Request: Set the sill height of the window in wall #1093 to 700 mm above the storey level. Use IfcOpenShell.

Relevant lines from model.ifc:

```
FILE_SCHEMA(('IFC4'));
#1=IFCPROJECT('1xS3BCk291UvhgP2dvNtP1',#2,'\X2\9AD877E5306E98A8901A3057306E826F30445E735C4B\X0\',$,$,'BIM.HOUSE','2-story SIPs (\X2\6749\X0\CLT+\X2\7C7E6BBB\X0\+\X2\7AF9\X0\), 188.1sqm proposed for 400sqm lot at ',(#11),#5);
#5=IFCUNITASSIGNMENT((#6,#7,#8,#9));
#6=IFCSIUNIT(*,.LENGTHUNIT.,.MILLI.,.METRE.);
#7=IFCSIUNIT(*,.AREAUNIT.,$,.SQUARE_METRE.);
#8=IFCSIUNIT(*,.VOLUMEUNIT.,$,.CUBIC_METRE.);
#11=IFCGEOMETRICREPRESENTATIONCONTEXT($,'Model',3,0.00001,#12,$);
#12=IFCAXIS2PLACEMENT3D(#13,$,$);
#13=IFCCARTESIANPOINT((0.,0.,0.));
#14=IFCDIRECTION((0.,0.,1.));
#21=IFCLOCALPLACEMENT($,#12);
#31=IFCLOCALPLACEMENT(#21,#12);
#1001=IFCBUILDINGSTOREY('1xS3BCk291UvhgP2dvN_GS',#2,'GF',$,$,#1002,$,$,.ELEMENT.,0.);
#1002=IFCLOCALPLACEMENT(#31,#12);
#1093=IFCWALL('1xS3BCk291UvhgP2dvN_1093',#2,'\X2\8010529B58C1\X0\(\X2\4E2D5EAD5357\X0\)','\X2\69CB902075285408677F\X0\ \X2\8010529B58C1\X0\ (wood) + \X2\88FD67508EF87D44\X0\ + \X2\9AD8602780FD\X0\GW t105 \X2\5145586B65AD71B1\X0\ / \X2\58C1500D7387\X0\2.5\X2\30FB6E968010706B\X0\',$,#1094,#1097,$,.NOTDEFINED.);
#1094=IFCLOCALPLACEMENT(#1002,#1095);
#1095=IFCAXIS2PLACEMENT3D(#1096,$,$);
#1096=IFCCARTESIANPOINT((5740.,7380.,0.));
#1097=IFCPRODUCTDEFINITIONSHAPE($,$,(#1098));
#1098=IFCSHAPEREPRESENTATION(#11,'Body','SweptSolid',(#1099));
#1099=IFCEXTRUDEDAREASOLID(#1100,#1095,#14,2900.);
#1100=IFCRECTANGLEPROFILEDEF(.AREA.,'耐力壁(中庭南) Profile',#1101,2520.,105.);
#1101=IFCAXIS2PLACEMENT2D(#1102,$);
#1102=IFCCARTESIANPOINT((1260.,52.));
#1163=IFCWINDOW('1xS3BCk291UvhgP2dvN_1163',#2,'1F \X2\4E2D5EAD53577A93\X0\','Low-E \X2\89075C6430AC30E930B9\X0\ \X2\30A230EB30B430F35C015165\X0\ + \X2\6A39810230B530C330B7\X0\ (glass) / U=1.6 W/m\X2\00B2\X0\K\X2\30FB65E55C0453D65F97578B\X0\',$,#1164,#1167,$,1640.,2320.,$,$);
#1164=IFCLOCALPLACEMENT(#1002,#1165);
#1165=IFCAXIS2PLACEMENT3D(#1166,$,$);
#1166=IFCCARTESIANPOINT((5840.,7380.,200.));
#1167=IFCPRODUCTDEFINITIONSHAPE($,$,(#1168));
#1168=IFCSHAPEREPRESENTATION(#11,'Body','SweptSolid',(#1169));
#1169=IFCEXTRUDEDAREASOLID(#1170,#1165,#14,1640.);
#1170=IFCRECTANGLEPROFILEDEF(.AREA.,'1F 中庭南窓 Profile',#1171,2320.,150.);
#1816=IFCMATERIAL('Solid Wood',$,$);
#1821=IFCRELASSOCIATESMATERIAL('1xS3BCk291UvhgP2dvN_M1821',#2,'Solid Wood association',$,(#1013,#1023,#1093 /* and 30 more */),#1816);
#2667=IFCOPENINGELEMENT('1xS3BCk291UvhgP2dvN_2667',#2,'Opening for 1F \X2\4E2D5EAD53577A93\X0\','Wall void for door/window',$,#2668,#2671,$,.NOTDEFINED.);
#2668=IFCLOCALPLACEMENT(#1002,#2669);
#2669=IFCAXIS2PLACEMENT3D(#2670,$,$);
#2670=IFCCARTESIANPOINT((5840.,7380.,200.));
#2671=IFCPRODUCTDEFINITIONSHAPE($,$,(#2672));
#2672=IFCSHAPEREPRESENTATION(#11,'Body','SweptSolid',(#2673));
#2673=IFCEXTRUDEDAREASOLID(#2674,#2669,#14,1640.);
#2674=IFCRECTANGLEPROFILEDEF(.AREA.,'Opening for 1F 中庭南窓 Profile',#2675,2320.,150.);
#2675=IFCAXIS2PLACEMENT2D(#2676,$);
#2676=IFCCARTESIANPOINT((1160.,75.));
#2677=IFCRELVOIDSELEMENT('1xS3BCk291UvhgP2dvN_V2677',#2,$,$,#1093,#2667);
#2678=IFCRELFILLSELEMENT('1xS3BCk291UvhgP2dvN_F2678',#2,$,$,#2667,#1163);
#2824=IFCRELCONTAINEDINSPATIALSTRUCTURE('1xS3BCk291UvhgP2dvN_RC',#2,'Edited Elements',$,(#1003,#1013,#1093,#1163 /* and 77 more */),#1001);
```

```python
import numpy as np
import ifcopenshell
import ifcopenshell.api.geometry
import ifcopenshell.geom
import ifcopenshell.util.element
import ifcopenshell.util.placement
import ifcopenshell.util.shape
import ifcopenshell.util.unit

model = ifcopenshell.open("model.ifc")
unit_scale = ifcopenshell.util.unit.calculate_unit_scale(model)

window = model.by_guid("1xS3BCk291UvhgP2dvN_1163")
opening = window.FillsVoids[0].RelatingOpeningElement
storey = ifcopenshell.util.element.get_container(window, ifc_class="IfcBuildingStorey")
level = ifcopenshell.util.placement.get_local_placement(storey.ObjectPlacement)[2, 3]

# The opening's origin need not be at the sill, so measure its lowest point.
shape = ifcopenshell.geom.create_shape(ifcopenshell.geom.settings(), opening)
bottom = ifcopenshell.util.shape.get_shape_bottom_elevation(shape, shape.geometry) / unit_scale
dz = level + 0.7 / unit_scale - bottom

shift = np.array([0.0, 0.0, dz])
# The window is not placed relative to its opening, so move both.
for product in (opening, window):
    matrix = ifcopenshell.util.placement.get_local_placement(product.ObjectPlacement)
    matrix[:3, 3] += shift
    ifcopenshell.api.geometry.edit_object_placement(model, product=product, matrix=matrix, is_si=False)

print(f"moved by {dz * unit_scale:+.3f} m")

model.write("model_edited.ifc")
```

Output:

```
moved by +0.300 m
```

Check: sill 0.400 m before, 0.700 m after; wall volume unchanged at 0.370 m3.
